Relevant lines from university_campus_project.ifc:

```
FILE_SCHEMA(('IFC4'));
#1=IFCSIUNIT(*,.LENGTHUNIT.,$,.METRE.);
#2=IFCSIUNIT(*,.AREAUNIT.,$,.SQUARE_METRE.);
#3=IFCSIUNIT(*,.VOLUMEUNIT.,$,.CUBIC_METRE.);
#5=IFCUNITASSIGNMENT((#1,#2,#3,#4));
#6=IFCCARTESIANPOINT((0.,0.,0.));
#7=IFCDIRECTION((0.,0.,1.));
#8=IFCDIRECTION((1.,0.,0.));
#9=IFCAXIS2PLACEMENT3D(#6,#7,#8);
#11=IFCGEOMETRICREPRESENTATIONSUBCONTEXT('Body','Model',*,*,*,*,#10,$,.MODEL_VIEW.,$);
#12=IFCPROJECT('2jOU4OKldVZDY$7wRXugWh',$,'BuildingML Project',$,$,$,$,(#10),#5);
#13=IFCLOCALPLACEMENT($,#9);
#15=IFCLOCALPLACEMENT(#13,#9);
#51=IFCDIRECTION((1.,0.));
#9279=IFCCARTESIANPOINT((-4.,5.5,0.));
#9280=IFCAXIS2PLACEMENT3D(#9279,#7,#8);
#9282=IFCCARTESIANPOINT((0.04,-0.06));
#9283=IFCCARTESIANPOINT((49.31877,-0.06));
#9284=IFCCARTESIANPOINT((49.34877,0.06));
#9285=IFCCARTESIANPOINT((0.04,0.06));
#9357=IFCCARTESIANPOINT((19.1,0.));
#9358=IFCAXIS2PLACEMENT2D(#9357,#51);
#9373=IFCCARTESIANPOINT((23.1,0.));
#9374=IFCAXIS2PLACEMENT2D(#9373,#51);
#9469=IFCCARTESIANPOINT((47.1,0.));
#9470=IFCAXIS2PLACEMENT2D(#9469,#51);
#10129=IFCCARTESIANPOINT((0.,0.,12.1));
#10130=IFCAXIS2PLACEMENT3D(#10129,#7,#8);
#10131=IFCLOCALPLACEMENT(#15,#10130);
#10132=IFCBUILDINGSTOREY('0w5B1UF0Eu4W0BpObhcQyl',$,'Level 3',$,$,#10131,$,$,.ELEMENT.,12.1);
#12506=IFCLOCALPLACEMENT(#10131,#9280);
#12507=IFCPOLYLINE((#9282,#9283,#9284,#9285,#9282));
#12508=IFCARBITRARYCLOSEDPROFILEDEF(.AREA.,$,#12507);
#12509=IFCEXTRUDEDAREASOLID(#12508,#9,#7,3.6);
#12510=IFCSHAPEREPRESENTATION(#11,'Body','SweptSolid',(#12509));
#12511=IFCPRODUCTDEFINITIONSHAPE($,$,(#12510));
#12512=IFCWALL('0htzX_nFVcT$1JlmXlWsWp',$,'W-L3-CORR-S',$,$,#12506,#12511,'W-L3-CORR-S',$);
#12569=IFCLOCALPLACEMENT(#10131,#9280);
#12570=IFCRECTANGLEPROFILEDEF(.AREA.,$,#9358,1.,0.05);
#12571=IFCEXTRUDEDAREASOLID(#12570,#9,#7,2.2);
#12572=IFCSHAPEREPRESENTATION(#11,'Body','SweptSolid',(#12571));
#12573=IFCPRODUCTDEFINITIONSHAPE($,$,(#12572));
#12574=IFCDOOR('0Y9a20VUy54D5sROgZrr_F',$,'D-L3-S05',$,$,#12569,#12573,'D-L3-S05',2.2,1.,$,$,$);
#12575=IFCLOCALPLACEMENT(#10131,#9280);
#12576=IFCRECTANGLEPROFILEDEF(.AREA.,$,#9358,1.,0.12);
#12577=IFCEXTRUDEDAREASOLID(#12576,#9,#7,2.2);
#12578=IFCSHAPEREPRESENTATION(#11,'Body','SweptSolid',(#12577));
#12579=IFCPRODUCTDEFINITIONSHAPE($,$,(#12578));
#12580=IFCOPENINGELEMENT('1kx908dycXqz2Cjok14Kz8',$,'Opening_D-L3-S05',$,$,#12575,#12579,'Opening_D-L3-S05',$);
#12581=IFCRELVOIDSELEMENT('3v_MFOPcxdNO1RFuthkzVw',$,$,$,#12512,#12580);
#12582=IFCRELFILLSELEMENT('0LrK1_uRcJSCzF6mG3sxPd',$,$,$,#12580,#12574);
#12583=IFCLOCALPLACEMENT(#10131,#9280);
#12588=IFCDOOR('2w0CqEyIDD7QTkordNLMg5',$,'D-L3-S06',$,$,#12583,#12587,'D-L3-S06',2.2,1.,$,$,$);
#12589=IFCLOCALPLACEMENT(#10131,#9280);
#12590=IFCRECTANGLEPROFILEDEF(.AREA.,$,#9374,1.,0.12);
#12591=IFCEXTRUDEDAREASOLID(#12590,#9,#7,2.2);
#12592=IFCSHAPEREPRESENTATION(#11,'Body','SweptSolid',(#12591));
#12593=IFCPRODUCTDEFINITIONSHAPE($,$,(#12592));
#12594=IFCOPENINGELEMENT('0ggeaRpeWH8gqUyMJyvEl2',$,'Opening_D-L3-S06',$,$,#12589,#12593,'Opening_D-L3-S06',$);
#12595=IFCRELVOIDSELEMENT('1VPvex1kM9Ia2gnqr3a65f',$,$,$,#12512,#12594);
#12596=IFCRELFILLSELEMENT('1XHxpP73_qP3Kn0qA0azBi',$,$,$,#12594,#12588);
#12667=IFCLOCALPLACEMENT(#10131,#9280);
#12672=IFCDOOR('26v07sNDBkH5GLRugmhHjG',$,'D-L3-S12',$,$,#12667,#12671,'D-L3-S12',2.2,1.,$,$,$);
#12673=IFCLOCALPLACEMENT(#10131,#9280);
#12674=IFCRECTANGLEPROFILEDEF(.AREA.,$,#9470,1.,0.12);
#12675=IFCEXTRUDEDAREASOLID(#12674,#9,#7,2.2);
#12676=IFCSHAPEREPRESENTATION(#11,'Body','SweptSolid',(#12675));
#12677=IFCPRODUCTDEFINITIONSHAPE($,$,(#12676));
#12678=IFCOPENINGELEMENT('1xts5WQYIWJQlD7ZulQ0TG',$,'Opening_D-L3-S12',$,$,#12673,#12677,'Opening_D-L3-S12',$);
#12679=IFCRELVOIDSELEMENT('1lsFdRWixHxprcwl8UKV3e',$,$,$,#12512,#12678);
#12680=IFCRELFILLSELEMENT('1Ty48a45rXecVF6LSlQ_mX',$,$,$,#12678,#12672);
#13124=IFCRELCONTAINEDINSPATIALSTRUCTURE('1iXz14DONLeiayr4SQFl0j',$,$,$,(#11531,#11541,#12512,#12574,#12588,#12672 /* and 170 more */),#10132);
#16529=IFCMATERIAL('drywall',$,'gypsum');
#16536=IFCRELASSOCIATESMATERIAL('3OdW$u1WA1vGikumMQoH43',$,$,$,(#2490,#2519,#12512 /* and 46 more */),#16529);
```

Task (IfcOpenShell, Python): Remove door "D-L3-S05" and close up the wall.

```python
import ifcopenshell
import ifcopenshell.api.feature
import ifcopenshell.api.root
import ifcopenshell.geom
import ifcopenshell.util.shape

model = ifcopenshell.open("university_campus_project.ifc")
settings = ifcopenshell.geom.settings()


def volume(element):
    """Net volume in cubic metres, openings subtracted."""
    shape = ifcopenshell.geom.create_shape(settings, element)
    return ifcopenshell.util.shape.get_volume(shape.geometry)


door = model.by_guid("0Y9a20VUy54D5sROgZrr_F")
opening = door.FillsVoids[0].RelatingOpeningElement
wall = opening.VoidsElements[0].RelatingBuildingElement
before = volume(wall)

ifcopenshell.api.root.remove_product(model, product=door)
ifcopenshell.api.feature.remove_feature(model, feature=opening)

after = volume(wall)

print(f"wall volume {before:.3f} -> {after:.3f} m3")

model.write("university_campus_project_updated.ifc")
```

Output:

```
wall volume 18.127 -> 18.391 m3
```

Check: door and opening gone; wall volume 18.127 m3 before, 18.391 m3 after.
